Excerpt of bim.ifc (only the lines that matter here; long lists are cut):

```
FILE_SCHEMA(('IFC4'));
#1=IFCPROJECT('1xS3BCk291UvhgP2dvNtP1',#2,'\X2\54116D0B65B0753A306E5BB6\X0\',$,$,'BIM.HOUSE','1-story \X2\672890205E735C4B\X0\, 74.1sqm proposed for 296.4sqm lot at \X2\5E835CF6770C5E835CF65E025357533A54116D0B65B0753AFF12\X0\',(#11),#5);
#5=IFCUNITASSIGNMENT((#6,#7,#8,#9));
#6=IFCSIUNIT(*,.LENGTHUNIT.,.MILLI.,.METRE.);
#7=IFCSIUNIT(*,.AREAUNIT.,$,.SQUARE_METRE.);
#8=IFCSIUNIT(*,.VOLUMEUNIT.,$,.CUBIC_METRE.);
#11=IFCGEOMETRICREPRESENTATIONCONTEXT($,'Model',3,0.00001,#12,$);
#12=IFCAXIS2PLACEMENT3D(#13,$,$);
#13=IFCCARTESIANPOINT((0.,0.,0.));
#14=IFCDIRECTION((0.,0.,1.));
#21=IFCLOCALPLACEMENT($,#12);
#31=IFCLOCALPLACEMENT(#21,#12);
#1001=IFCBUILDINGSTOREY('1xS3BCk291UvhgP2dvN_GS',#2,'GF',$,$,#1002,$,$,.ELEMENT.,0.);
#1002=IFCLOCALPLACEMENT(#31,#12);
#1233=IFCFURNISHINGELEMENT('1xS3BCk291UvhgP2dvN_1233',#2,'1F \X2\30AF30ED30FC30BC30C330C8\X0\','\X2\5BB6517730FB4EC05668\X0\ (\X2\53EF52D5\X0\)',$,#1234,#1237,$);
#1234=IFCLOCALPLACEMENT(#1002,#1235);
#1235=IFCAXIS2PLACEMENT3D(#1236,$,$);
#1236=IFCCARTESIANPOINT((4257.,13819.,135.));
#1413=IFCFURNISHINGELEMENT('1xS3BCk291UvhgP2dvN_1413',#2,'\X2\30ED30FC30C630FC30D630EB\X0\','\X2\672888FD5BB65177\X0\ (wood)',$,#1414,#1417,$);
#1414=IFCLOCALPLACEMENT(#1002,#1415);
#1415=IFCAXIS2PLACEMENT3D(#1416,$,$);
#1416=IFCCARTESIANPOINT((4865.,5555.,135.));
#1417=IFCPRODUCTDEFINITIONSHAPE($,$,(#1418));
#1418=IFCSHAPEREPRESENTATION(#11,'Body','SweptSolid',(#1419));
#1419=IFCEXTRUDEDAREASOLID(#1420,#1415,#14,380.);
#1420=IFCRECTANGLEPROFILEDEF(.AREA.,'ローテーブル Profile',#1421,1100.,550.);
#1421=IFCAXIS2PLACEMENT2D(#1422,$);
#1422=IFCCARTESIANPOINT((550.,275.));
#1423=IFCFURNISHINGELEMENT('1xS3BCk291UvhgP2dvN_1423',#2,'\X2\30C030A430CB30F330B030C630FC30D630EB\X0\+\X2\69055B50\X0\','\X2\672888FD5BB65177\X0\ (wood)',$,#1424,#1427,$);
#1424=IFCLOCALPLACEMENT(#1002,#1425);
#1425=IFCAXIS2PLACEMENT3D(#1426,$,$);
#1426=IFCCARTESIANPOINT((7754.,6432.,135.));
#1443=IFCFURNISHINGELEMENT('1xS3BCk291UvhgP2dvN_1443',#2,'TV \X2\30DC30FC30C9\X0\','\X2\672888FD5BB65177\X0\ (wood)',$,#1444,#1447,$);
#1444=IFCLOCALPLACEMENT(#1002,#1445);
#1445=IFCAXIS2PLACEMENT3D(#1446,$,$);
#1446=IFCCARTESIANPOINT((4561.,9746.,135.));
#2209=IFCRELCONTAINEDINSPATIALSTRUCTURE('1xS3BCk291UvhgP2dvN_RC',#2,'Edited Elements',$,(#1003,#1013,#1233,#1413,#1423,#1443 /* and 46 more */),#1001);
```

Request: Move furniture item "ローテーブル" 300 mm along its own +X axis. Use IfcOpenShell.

```python
import ifcopenshell
import ifcopenshell.api.geometry
import ifcopenshell.util.placement

model = ifcopenshell.open("bim.ifc")

item = model.by_guid("1xS3BCk291UvhgP2dvN_1413")
matrix = ifcopenshell.util.placement.get_local_placement(item.ObjectPlacement)
matrix[:3, 3] += matrix[:3, 0] * 300.0
ifcopenshell.api.geometry.edit_object_placement(model, product=item, matrix=matrix, is_si=False)

print(ifcopenshell.util.placement.get_local_placement(item.ObjectPlacement).round(3) + 0.0)

model.write("bim_edited.ifc")
```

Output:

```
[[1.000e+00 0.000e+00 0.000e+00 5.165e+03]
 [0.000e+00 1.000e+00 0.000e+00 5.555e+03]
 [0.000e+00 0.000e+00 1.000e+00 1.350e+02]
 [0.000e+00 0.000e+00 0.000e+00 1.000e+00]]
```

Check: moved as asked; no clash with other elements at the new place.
